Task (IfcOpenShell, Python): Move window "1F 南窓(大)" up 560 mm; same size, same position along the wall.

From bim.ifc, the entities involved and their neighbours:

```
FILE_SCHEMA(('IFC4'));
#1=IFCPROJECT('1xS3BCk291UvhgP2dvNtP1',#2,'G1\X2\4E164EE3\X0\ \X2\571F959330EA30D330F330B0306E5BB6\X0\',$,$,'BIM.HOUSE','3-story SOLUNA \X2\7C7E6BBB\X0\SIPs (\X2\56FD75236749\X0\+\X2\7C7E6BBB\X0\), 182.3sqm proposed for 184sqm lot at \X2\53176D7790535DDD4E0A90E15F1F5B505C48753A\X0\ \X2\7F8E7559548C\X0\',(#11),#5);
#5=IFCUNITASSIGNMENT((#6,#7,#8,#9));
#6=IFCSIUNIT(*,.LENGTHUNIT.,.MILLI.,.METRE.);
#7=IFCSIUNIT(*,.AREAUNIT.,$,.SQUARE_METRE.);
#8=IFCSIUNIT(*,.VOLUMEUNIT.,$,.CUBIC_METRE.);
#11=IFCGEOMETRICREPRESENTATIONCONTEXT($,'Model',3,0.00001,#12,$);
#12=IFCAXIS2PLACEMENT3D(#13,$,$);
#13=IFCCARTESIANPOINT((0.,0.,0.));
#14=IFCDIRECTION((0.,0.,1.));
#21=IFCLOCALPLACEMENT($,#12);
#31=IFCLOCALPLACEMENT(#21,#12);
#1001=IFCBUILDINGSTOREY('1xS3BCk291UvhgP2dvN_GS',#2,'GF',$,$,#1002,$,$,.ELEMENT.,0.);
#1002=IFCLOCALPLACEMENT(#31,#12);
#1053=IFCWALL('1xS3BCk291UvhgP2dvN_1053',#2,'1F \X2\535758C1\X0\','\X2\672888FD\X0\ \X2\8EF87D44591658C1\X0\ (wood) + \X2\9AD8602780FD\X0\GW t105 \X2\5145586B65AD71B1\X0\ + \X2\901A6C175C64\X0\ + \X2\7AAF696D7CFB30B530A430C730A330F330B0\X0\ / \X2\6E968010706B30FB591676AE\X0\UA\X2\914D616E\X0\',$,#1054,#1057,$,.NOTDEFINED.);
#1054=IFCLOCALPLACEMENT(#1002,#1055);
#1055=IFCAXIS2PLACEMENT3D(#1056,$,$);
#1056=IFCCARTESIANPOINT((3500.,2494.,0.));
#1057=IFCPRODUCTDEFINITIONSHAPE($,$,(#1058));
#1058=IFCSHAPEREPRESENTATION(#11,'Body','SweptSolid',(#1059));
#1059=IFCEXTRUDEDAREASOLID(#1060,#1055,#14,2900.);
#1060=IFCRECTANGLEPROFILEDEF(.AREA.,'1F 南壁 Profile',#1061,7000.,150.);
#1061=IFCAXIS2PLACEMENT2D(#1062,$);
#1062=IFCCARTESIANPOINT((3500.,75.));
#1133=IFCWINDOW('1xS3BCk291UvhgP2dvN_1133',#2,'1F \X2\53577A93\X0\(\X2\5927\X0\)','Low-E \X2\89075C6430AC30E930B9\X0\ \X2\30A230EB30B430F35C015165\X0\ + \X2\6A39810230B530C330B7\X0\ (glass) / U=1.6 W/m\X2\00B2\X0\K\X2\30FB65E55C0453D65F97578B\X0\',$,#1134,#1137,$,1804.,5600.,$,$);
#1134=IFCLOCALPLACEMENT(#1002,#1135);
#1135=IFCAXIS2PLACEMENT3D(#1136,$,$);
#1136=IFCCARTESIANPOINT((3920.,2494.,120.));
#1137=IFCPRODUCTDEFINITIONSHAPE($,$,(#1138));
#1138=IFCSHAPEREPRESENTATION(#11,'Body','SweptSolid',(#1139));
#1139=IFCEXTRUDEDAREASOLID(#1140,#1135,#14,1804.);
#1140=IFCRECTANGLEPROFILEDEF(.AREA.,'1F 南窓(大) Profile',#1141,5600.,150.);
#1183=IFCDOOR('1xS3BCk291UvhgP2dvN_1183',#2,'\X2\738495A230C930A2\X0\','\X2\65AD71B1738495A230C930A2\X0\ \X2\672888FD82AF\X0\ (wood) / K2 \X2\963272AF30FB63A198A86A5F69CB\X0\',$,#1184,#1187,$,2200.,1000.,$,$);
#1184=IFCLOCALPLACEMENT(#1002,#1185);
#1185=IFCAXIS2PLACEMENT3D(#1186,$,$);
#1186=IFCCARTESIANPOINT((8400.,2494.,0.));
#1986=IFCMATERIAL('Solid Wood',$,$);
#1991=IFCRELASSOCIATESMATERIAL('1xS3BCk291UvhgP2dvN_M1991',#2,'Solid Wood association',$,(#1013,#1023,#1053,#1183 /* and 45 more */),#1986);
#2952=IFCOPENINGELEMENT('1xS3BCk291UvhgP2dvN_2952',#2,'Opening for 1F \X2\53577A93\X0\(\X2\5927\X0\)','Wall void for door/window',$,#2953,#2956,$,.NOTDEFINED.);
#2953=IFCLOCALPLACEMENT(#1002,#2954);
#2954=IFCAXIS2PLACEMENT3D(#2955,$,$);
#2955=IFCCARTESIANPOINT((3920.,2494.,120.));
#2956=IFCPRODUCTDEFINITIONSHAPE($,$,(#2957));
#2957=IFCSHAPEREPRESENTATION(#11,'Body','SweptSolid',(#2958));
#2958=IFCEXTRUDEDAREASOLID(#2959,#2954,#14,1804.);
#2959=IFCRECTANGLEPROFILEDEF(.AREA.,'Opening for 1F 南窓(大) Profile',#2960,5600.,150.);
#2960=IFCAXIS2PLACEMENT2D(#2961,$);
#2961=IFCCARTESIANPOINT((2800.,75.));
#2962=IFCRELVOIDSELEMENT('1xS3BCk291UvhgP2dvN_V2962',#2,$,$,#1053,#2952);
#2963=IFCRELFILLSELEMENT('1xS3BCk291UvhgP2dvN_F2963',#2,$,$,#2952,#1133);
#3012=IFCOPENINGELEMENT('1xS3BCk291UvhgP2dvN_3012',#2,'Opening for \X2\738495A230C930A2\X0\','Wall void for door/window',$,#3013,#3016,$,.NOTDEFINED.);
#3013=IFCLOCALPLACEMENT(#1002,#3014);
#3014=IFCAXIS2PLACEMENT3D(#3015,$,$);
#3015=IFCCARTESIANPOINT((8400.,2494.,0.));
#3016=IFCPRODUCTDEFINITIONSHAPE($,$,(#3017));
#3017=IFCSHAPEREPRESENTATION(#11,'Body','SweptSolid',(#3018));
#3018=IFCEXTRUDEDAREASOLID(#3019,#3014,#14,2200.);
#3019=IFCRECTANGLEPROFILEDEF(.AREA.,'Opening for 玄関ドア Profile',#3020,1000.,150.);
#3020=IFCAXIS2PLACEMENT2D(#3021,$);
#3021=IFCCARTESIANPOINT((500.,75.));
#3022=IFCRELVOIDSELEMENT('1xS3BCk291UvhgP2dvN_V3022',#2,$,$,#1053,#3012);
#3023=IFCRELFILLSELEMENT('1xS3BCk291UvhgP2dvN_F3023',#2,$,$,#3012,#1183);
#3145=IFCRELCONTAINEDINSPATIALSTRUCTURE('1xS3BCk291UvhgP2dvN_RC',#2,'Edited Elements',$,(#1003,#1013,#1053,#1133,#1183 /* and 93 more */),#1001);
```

```python
import numpy as np
import ifcopenshell
import ifcopenshell.api.geometry
import ifcopenshell.util.placement
import ifcopenshell.util.unit

model = ifcopenshell.open("bim.ifc")
unit_scale = ifcopenshell.util.unit.calculate_unit_scale(model)

window = model.by_id(1133)
opening = window.FillsVoids[0].RelatingOpeningElement
dz = 0.56 / unit_scale

shift = np.array([0.0, 0.0, dz])
# The window is not placed relative to its opening, so move both.
for product in (opening, window):
    matrix = ifcopenshell.util.placement.get_local_placement(product.ObjectPlacement)
    matrix[:3, 3] += shift
    ifcopenshell.api.geometry.edit_object_placement(model, product=product, matrix=matrix, is_si=False)

print(f"moved by {dz * unit_scale:+.3f} m")

model.write("bim_rev.ifc")
```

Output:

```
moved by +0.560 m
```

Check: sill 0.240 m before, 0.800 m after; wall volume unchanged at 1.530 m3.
